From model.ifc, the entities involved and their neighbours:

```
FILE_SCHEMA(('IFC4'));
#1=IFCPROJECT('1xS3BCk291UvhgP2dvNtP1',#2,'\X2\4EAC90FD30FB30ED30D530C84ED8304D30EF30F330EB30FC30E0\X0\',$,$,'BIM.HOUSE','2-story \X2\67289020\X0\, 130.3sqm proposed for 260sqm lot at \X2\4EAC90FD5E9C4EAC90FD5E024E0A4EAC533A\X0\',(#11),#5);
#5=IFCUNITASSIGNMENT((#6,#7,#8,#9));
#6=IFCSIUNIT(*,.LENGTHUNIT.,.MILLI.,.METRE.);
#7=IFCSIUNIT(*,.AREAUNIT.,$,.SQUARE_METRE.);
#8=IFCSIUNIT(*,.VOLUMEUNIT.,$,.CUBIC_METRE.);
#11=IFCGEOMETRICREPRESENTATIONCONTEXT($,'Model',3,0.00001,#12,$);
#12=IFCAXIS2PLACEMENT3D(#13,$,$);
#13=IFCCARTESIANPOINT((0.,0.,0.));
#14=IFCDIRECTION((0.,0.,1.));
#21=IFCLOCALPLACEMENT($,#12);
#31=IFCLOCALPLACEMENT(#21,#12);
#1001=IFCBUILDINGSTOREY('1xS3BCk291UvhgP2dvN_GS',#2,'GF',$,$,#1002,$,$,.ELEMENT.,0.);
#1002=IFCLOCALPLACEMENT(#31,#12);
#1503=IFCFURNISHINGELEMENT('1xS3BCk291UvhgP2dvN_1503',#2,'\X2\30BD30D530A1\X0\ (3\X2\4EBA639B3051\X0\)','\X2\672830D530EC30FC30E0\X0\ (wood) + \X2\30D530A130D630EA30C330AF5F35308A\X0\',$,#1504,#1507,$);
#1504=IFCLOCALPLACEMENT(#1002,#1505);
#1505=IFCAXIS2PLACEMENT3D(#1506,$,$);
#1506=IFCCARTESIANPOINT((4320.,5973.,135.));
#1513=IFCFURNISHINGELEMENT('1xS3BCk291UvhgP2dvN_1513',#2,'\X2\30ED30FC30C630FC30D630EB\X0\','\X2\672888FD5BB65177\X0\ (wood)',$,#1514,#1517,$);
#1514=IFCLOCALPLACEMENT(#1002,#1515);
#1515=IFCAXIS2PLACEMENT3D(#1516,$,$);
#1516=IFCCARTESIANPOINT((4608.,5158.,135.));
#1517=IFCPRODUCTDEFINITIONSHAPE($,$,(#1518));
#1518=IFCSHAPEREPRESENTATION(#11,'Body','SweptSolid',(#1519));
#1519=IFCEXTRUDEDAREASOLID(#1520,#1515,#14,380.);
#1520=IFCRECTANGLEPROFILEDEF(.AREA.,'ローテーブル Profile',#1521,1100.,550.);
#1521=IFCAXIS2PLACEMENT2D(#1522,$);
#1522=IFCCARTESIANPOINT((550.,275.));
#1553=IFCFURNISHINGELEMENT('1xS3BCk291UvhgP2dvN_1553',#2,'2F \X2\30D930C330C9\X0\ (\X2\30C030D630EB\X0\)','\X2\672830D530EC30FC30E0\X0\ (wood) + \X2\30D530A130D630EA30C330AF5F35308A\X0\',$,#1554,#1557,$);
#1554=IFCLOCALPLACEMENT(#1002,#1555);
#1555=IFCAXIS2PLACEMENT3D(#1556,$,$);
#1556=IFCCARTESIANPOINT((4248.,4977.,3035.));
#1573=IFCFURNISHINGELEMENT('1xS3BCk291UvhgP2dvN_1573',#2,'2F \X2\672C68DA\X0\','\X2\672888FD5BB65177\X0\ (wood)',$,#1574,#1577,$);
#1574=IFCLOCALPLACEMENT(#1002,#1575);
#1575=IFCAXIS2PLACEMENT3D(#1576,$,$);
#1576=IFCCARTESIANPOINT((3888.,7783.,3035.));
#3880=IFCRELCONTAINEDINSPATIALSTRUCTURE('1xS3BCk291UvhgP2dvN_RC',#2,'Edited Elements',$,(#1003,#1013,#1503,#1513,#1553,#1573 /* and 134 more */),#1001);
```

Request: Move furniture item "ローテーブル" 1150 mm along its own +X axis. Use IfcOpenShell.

```python
import ifcopenshell
import ifcopenshell.api.geometry
import ifcopenshell.util.placement
import ifcopenshell.util.unit

model = ifcopenshell.open("model.ifc")
unit_scale = ifcopenshell.util.unit.calculate_unit_scale(model)

item = model.by_guid("1xS3BCk291UvhgP2dvN_1513")
matrix = ifcopenshell.util.placement.get_local_placement(item.ObjectPlacement)
matrix[:3, 3] += matrix[:3, 0] * 1.15 / unit_scale
ifcopenshell.api.geometry.edit_object_placement(model, product=item, matrix=matrix, is_si=False)

print(ifcopenshell.util.placement.get_local_placement(item.ObjectPlacement).round(3) + 0.0)

model.write("model_rev.ifc")
```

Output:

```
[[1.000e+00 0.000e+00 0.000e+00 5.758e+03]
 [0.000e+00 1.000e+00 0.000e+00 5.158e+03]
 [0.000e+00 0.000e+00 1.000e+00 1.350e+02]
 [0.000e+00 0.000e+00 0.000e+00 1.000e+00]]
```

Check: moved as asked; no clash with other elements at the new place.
